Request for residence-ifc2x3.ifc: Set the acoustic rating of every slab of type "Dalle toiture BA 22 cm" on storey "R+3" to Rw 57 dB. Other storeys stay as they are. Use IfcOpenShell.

First a look at what the model holds.

```python
import ifcopenshell
import ifcopenshell.util.element

model = ifcopenshell.open("residence-ifc2x3.ifc")
print(model.schema)
storey = next(s for s in model.by_type("IfcBuildingStorey") if s.Name == "R+3")
slabs = [e for e in ifcopenshell.util.element.get_decomposition(storey) if e.is_a("IfcSlab")]
seen = {}
for e in slabs:
    element_type = ifcopenshell.util.element.get_type(e)
    key = (element_type.Name if element_type != e and element_type else None, ifcopenshell.util.element.get_pset(e, "Pset_SlabCommon", "AcousticRating"))
    seen[key] = seen.get(key, 0) + 1
for (name, value), count in sorted(seen.items(), key=str):
    print(count, "x", name, "|", value)
```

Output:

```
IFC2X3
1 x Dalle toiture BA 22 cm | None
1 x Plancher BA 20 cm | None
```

```python
import ifcopenshell
import ifcopenshell.api.pset
import ifcopenshell.util.element

model = ifcopenshell.open("residence-ifc2x3.ifc")

storey = next(s for s in model.by_type("IfcBuildingStorey") if s.Name == "R+3")
slabs = [e for e in ifcopenshell.util.element.get_decomposition(storey) if e.is_a("IfcSlab")]

count = 0
for e in slabs:
    element_type = ifcopenshell.util.element.get_type(e)
    if element_type in (None, e) or element_type.Name != "Dalle toiture BA 22 cm":
        continue
    # add_pset returns the element's existing set when there is one.
    pset = ifcopenshell.api.pset.add_pset(model, product=e, name="Pset_SlabCommon")
    ifcopenshell.api.pset.edit_pset(model, pset=pset, properties={"AcousticRating": "Rw 57 dB"})
    count += 1

print(count, "slabs updated")

model.write("residence-ifc2x3_edited.ifc")
```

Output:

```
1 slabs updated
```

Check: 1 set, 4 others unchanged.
